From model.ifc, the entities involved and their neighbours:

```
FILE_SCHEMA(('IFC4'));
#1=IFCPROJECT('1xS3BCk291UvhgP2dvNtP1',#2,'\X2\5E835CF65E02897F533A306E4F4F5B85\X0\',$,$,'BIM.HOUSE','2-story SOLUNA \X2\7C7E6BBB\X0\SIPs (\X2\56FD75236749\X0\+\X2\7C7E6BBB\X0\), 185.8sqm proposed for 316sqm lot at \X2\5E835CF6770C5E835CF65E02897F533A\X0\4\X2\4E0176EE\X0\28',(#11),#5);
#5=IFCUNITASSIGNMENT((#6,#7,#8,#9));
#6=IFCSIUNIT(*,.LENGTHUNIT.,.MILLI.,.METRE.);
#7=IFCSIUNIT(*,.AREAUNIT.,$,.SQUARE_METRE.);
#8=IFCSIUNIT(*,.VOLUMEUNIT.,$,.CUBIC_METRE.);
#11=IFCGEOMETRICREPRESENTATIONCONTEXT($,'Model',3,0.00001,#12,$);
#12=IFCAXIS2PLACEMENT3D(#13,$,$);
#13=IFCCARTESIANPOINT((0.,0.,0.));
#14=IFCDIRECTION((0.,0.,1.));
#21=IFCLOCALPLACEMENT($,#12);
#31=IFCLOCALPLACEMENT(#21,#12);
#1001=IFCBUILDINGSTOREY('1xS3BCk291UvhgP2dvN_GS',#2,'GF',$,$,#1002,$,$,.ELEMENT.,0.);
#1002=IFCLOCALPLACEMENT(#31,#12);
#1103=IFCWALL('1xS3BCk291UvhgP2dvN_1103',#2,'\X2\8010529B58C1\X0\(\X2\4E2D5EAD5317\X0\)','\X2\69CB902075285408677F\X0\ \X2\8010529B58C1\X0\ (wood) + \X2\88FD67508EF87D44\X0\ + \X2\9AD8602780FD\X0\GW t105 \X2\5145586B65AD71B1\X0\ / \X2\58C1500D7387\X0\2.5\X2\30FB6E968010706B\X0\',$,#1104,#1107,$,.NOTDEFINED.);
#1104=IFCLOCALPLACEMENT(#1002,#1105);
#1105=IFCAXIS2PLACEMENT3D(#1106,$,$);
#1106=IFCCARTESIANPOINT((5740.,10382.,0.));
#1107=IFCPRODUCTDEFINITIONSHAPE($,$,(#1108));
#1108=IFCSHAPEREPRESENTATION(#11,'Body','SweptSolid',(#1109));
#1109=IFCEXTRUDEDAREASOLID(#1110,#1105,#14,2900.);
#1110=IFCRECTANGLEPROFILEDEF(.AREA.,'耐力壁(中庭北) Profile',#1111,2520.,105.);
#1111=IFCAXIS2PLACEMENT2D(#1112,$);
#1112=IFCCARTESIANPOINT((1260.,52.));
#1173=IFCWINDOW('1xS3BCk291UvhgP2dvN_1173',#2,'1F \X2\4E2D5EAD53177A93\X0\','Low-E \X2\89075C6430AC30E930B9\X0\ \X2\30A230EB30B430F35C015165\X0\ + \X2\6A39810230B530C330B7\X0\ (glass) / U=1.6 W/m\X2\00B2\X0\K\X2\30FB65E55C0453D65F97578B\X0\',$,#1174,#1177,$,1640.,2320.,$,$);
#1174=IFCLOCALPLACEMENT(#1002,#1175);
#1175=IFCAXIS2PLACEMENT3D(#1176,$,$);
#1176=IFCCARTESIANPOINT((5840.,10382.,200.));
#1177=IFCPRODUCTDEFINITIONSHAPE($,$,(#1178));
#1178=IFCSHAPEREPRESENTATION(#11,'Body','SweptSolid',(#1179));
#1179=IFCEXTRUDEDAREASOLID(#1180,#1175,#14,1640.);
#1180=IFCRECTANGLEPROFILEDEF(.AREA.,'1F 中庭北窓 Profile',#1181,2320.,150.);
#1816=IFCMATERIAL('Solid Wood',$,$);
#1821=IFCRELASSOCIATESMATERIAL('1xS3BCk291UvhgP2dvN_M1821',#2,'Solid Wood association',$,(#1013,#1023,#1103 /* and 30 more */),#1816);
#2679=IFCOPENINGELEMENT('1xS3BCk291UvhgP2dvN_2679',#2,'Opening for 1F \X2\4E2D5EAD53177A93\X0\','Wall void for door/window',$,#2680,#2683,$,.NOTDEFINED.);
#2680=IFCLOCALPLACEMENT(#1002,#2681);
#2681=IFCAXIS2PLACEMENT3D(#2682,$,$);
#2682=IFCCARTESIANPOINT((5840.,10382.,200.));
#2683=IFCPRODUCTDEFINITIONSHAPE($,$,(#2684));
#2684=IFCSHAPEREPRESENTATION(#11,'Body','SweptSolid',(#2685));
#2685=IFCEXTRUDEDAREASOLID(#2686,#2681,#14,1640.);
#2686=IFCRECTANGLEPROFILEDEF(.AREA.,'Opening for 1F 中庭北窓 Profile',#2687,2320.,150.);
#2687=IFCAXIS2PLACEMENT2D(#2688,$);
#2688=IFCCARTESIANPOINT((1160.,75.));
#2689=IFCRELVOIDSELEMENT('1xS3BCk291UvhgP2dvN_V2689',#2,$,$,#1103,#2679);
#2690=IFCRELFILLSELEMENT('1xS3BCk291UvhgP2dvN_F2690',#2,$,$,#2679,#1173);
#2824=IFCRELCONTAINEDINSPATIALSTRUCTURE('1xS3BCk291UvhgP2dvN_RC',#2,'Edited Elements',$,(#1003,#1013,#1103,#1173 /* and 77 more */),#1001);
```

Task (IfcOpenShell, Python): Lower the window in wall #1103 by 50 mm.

```python
import numpy as np
import ifcopenshell
import ifcopenshell.api.geometry
import ifcopenshell.util.placement
import ifcopenshell.util.unit

model = ifcopenshell.open("model.ifc")
unit_scale = ifcopenshell.util.unit.calculate_unit_scale(model)

window = model.by_guid("1xS3BCk291UvhgP2dvN_1173")
opening = window.FillsVoids[0].RelatingOpeningElement
dz = -50.0

shift = np.array([0.0, 0.0, dz])
# The window is not placed relative to its opening, so move both.
for product in (opening, window):
    matrix = ifcopenshell.util.placement.get_local_placement(product.ObjectPlacement)
    matrix[:3, 3] += shift
    ifcopenshell.api.geometry.edit_object_placement(model, product=product, matrix=matrix, is_si=False)

print(f"moved by {dz * unit_scale:+.3f} m")

model.write("model_updated.ifc")
```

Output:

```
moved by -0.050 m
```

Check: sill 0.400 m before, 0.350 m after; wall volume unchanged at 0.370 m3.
